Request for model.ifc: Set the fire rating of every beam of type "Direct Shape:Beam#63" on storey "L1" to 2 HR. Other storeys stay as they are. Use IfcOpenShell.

First a look at what the model holds.

```python
import ifcopenshell
import ifcopenshell.util.element

model = ifcopenshell.open("model.ifc")
print(model.schema)
storey = next(s for s in model.by_type("IfcBuildingStorey") if s.Name == "L1")
beams = [e for e in ifcopenshell.util.element.get_decomposition(storey) if e.is_a("IfcBeam")]
seen = {}
for e in beams:
    element_type = ifcopenshell.util.element.get_type(e)
    key = (element_type.Name if element_type != e and element_type else None, ifcopenshell.util.element.get_pset(e, "Pset_BeamCommon", "FireRating"))
    seen[key] = seen.get(key, 0) + 1
for (name, value), count in sorted(seen.items(), key=str):
    print(count, "x", name, "|", value)
```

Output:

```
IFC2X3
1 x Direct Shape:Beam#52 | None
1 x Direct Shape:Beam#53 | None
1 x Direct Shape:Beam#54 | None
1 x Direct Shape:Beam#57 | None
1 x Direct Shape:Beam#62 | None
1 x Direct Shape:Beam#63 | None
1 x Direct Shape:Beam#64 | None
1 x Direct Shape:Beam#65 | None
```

```python
import ifcopenshell
import ifcopenshell.api.pset
import ifcopenshell.util.element

model = ifcopenshell.open("model.ifc")

storey = next(s for s in model.by_type("IfcBuildingStorey") if s.Name == "L1")
beams = [e for e in ifcopenshell.util.element.get_decomposition(storey) if e.is_a("IfcBeam")]

count = 0
for e in beams:
    element_type = ifcopenshell.util.element.get_type(e)
    if element_type in (None, e) or element_type.Name != "Direct Shape:Beam#63":
        continue
    # add_pset returns the element's existing set when there is one.
    pset = ifcopenshell.api.pset.add_pset(model, product=e, name="Pset_BeamCommon")
    ifcopenshell.api.pset.edit_pset(model, pset=pset, properties={"FireRating": "2 HR"})
    count += 1

print(count, "beams updated")

model.write("model_rev.ifc")
```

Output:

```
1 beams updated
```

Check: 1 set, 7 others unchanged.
